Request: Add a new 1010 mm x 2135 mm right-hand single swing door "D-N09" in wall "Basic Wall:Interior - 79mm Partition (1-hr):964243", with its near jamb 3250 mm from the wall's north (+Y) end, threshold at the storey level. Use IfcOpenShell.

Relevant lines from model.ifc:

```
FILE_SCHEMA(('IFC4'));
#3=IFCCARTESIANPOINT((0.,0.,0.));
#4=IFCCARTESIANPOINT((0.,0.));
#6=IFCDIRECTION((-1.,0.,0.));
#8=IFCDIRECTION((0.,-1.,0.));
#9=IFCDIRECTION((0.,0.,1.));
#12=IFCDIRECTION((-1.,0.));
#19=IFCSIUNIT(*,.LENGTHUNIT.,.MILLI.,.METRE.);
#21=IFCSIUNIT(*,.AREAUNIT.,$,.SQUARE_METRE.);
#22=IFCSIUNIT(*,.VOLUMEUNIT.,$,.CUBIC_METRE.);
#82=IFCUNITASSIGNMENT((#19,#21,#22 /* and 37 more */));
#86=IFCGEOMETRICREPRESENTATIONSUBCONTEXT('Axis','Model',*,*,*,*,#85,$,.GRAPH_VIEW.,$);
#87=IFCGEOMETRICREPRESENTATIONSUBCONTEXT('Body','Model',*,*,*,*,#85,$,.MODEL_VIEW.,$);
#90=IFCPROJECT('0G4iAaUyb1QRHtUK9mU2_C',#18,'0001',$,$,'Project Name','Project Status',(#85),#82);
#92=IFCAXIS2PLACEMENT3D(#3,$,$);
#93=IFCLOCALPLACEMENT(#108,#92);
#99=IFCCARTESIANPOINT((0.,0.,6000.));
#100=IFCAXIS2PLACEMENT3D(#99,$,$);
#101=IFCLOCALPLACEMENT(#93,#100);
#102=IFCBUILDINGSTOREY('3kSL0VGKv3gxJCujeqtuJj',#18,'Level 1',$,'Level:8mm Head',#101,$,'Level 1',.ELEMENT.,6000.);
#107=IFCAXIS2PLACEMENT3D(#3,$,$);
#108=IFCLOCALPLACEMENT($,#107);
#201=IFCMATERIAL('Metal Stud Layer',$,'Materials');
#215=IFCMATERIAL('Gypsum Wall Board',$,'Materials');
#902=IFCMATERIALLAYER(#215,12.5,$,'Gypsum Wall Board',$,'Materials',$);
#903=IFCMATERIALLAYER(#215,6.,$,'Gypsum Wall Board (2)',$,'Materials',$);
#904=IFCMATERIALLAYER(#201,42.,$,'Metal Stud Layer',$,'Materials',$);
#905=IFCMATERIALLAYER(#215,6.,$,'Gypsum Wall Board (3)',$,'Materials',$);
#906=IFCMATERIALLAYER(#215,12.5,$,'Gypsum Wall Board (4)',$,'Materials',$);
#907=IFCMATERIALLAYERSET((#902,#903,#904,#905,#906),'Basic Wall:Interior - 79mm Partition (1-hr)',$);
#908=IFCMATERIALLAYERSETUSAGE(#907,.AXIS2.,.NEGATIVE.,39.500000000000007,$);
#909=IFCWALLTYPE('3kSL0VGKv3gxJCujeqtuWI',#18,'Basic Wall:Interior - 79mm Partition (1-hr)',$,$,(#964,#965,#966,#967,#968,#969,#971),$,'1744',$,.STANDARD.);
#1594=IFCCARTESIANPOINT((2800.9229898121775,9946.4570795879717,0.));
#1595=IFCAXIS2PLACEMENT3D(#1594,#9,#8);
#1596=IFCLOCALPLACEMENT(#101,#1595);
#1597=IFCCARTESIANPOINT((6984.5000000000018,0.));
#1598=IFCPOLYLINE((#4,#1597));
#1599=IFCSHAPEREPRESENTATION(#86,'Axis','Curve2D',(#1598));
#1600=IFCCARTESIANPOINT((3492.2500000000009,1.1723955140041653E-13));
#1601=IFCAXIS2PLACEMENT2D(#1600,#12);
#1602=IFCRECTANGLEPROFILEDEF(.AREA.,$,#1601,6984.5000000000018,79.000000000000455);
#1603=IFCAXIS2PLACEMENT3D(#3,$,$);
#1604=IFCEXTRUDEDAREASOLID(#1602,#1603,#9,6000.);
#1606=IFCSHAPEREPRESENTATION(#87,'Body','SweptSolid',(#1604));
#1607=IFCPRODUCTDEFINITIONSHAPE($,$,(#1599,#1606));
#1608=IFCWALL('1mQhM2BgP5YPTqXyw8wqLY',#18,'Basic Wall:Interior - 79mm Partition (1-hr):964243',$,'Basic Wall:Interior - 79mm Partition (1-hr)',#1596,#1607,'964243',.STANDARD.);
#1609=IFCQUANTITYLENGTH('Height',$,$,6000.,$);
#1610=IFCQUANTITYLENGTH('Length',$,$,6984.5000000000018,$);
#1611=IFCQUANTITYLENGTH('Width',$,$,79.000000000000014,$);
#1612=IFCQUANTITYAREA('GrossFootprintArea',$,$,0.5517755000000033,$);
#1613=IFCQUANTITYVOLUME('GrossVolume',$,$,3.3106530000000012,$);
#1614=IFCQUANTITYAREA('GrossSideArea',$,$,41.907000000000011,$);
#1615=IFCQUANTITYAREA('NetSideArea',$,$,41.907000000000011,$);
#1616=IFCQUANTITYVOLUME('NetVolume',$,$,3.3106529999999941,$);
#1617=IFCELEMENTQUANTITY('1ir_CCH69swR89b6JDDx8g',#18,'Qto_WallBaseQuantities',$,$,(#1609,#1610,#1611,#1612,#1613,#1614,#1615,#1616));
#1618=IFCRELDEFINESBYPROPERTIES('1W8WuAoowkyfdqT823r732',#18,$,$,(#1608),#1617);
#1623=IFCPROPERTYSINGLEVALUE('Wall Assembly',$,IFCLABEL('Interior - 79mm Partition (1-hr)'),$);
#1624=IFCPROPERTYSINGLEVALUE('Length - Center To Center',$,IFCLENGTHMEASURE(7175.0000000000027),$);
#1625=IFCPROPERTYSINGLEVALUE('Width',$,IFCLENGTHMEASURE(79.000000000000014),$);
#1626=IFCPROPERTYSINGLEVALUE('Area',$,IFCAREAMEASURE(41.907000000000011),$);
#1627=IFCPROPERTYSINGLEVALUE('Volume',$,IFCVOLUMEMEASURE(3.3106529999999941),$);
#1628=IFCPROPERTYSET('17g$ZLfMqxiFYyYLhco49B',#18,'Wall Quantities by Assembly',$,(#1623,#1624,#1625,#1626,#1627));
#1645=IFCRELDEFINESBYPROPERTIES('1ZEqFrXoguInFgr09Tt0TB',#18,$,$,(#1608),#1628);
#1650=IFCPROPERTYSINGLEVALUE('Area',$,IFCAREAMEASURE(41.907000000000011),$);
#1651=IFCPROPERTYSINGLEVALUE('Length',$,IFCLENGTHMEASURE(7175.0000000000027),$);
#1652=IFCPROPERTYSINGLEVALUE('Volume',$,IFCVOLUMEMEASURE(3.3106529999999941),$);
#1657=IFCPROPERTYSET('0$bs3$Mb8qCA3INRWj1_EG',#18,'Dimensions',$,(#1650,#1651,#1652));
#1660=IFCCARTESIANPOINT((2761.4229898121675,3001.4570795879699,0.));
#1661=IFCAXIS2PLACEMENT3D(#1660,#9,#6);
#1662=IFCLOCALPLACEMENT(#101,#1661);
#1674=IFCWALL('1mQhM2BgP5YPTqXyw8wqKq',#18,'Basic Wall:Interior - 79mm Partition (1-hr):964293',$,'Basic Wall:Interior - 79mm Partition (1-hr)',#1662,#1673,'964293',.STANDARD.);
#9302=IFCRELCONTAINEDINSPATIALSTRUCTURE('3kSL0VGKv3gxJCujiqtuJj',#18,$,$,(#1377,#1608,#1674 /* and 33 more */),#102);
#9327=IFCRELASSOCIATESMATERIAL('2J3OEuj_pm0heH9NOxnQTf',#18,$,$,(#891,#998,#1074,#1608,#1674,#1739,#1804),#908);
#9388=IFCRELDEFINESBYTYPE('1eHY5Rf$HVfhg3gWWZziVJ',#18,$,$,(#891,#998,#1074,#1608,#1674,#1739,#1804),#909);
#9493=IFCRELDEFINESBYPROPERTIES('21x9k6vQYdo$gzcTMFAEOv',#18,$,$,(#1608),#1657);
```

```python
import numpy as np
import ifcopenshell
import ifcopenshell.api.feature
import ifcopenshell.api.geometry
import ifcopenshell.api.pset
import ifcopenshell.api.root
import ifcopenshell.api.spatial
import ifcopenshell.geom
import ifcopenshell.util.element
import ifcopenshell.util.placement
import ifcopenshell.util.representation
import ifcopenshell.util.shape
import ifcopenshell.util.unit

model = ifcopenshell.open("model.ifc")
unit_scale = ifcopenshell.util.unit.calculate_unit_scale(model)
area_scale = ifcopenshell.util.unit.calculate_unit_scale(model, "AREAUNIT")
volume_scale = ifcopenshell.util.unit.calculate_unit_scale(model, "VOLUMEUNIT")
settings = ifcopenshell.geom.settings()


def volume(element):
    """Net volume in cubic metres, openings subtracted."""
    shape = ifcopenshell.geom.create_shape(settings, element)
    return ifcopenshell.util.shape.get_volume(shape.geometry)


wall = model.by_guid("1mQhM2BgP5YPTqXyw8wqLY")
storey = ifcopenshell.util.element.get_container(wall, ifc_class="IfcBuildingStorey")
context = ifcopenshell.util.representation.get_context(model, "Model", "Body", "MODEL_VIEW")
before = volume(wall)

width, height, from_end, sill = 1.01, 2.135, 3.25, 0.0  # metres

# The wall runs along its own X axis, and the end named is its -X end.
wall_shape = ifcopenshell.geom.create_shape(settings, wall)
x, y, z = ifcopenshell.util.shape.get_vertices(wall_shape.geometry).T
start = x.min() + from_end
face, thickness = float(y.min()), float(y.max() - y.min())
wall_matrix = ifcopenshell.util.placement.get_local_placement(wall.ObjectPlacement)
level = ifcopenshell.util.placement.get_local_placement(storey.ObjectPlacement)[2, 3]


def in_wall(x, y):
    """Placement at x, y metres in the wall's axes, at sill height."""
    matrix = wall_matrix.copy()
    matrix[:, 3] = wall_matrix @ np.array([x / unit_scale, y / unit_scale, 0.0, 1.0])
    matrix[2, 3] = level + sill / unit_scale
    return matrix


# Opening: a box that overshoots both wall faces by 50 mm.
opening = ifcopenshell.api.root.create_entity(model, ifc_class="IfcOpeningElement", predefined_type="OPENING")
box = ifcopenshell.api.geometry.add_wall_representation(
    model, context=context, length=width, height=height, thickness=thickness + 0.1
)
ifcopenshell.api.geometry.assign_representation(model, product=opening, representation=box)
ifcopenshell.api.geometry.edit_object_placement(model, product=opening, matrix=in_wall(start, face - 0.05), is_si=False)
ifcopenshell.api.feature.add_feature(model, feature=opening, element=wall)

door = ifcopenshell.api.root.create_entity(model, ifc_class="IfcDoor", name="D-N09", predefined_type="DOOR")
door.OverallWidth, door.OverallHeight = width / unit_scale, height / unit_scale
door.OperationType = "SINGLE_SWING_RIGHT"
body = ifcopenshell.api.geometry.add_door_representation(
    model,
    context=context,
    overall_width=door.OverallWidth,
    overall_height=door.OverallHeight,
    operation_type="SINGLE_SWING_RIGHT",
    lining_properties={"LiningDepth": thickness / unit_scale, "ThresholdDepth": thickness / unit_scale},
)
ifcopenshell.api.geometry.assign_representation(model, product=door, representation=body)
ifcopenshell.api.spatial.assign_container(model, products=[door], relating_structure=storey)
ifcopenshell.api.feature.add_filling(model, opening=opening, element=door)

# The lining spans the wall, so the door starts at the wall face.
ifcopenshell.api.geometry.edit_object_placement(model, product=door, matrix=in_wall(start, face), is_si=False)

after = volume(wall)

# Update the wall's stored quantities.
qto = model.by_id(ifcopenshell.util.element.get_pset(wall, "Qto_WallBaseQuantities", should_inherit=False)["id"])
ifcopenshell.api.pset.edit_qto(model, qto=qto, properties={
    "NetSideArea": after / thickness / area_scale,
    "NetVolume": after / volume_scale,
})
pset = model.by_id(ifcopenshell.util.element.get_pset(wall, "Wall Quantities by Assembly", should_inherit=False)["id"])
ifcopenshell.api.pset.edit_pset(model, pset=pset, properties={
    "Area": model.create_entity("IfcAreaMeasure", after / thickness / area_scale),
    "Volume": model.create_entity("IfcVolumeMeasure", after / volume_scale),
})
pset = model.by_id(ifcopenshell.util.element.get_pset(wall, "Dimensions", should_inherit=False)["id"])
ifcopenshell.api.pset.edit_pset(model, pset=pset, properties={
    "Area": model.create_entity("IfcAreaMeasure", after / thickness / area_scale),
    "Volume": model.create_entity("IfcVolumeMeasure", after / volume_scale),
})

print(f"wall volume {before:.3f} -> {after:.3f} m3")

model.write("model_updated.ifc")
```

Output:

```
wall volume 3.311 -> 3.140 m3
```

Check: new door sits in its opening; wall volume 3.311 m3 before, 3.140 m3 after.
